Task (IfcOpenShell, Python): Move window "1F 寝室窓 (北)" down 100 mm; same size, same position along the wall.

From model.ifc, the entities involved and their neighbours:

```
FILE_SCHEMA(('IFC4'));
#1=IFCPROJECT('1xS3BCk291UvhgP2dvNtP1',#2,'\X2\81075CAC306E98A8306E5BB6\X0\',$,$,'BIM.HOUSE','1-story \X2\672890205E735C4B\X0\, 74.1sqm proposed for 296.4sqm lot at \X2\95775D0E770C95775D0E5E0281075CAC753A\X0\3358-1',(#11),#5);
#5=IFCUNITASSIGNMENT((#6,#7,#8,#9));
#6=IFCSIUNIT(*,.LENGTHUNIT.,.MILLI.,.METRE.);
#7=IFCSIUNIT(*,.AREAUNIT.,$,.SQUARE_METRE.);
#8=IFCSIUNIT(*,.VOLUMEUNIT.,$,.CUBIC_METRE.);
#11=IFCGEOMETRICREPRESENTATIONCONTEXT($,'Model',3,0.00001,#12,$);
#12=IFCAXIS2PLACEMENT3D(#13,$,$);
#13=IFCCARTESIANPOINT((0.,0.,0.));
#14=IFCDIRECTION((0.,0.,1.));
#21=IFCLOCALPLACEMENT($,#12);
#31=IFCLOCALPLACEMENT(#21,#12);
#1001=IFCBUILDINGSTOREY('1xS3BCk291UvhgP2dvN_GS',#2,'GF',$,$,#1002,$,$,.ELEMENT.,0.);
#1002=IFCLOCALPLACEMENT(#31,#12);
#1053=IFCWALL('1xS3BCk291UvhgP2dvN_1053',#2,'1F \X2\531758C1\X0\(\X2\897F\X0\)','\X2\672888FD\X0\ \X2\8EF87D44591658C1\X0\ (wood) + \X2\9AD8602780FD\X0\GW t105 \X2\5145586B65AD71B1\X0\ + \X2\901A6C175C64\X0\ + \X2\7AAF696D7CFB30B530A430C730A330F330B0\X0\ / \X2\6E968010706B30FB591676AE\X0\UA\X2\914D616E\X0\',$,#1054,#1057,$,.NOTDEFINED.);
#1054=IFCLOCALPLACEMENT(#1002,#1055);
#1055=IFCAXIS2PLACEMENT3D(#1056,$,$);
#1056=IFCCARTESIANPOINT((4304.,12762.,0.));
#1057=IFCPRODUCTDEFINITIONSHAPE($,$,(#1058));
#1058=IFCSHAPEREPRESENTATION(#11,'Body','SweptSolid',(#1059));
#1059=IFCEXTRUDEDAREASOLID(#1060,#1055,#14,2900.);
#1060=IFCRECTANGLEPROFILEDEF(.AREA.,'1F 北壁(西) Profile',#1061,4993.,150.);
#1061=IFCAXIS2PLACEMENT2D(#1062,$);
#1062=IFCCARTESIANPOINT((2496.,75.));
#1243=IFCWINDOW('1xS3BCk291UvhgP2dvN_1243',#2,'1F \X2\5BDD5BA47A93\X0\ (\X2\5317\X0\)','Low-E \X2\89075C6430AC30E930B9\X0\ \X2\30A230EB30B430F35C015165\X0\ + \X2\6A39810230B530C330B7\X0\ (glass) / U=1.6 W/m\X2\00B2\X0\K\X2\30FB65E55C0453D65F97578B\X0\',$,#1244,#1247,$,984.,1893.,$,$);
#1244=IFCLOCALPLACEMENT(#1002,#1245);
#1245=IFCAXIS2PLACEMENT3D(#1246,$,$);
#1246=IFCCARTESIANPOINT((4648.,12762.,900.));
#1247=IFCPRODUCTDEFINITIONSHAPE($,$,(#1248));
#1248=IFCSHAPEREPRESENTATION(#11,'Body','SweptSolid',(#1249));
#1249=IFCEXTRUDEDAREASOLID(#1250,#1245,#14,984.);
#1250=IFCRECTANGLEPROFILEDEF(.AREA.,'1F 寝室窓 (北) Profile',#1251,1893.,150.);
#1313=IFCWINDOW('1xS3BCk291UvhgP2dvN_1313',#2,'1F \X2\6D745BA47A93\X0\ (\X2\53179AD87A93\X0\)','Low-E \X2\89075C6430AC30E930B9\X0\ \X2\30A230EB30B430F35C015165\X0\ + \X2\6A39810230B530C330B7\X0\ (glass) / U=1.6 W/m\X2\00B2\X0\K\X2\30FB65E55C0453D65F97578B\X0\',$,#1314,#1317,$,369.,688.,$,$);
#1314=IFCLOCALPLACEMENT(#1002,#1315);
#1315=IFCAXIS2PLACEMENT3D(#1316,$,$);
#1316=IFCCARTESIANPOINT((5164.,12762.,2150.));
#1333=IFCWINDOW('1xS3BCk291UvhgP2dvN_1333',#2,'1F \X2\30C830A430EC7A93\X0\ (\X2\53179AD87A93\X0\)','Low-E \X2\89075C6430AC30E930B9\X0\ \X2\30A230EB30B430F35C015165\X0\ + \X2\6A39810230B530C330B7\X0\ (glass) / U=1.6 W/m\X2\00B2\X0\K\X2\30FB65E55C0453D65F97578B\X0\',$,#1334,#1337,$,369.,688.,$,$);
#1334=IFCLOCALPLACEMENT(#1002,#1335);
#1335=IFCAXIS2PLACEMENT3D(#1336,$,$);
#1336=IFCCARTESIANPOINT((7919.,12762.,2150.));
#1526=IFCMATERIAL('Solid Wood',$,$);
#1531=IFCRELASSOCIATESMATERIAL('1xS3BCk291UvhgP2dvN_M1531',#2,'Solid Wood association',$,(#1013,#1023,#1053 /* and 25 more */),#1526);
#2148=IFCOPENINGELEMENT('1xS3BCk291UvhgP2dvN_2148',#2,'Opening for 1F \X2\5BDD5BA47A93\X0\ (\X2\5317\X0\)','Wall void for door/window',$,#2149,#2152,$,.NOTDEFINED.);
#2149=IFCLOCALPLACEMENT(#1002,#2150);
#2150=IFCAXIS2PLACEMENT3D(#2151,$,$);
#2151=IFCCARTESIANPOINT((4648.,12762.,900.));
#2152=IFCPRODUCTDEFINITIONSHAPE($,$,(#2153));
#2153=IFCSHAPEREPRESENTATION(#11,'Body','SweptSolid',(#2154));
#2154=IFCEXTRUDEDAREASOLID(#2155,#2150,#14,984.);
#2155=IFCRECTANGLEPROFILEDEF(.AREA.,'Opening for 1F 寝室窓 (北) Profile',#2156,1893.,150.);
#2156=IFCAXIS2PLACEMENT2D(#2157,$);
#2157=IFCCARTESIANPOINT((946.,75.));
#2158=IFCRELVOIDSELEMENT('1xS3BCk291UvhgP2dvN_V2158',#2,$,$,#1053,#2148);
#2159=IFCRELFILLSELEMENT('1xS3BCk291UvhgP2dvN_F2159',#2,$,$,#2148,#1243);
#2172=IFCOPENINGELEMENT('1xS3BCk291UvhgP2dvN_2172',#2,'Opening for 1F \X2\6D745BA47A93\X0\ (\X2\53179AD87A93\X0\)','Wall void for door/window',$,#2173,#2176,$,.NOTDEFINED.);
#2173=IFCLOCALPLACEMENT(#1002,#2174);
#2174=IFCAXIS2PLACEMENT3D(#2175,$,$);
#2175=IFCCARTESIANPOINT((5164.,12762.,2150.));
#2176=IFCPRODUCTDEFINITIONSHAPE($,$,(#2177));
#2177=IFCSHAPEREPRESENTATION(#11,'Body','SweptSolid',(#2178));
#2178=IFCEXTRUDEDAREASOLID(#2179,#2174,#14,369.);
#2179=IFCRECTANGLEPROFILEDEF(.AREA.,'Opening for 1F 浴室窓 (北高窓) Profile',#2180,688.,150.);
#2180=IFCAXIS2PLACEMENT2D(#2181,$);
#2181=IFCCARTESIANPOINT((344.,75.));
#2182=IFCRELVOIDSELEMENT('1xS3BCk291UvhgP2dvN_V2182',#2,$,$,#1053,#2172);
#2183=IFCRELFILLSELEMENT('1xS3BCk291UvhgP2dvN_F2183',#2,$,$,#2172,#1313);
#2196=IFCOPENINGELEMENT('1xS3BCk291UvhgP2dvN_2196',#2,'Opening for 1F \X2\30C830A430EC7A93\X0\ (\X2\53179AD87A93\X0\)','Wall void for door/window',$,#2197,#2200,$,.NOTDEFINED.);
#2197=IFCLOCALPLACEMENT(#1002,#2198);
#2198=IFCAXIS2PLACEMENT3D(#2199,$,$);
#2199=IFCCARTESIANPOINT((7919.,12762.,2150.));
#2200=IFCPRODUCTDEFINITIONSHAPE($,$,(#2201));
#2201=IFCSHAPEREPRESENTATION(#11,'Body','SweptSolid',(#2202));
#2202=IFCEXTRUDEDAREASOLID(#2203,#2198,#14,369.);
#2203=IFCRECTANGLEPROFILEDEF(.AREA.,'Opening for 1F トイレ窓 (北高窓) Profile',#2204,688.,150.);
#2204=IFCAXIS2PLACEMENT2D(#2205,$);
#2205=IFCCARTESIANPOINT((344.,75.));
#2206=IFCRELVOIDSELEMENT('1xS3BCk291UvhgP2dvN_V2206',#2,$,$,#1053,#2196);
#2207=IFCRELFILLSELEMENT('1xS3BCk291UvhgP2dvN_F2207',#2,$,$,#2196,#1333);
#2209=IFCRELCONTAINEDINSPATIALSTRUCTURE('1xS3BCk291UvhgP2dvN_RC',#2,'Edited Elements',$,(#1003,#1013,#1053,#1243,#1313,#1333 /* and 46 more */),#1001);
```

```python
import numpy as np
import ifcopenshell
import ifcopenshell.api.geometry
import ifcopenshell.util.placement
import ifcopenshell.util.unit

model = ifcopenshell.open("model.ifc")
unit_scale = ifcopenshell.util.unit.calculate_unit_scale(model)

window = model.by_id(1243)
opening = window.FillsVoids[0].RelatingOpeningElement
dz = -0.1 / unit_scale

shift = np.array([0.0, 0.0, dz])
# The window is not placed relative to its opening, so move both.
for product in (opening, window):
    matrix = ifcopenshell.util.placement.get_local_placement(product.ObjectPlacement)
    matrix[:3, 3] += shift
    ifcopenshell.api.geometry.edit_object_placement(model, product=product, matrix=matrix, is_si=False)

print(f"moved by {dz * unit_scale:+.3f} m")

model.write("model-out.ifc")
```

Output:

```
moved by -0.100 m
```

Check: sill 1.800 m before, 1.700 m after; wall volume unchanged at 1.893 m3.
